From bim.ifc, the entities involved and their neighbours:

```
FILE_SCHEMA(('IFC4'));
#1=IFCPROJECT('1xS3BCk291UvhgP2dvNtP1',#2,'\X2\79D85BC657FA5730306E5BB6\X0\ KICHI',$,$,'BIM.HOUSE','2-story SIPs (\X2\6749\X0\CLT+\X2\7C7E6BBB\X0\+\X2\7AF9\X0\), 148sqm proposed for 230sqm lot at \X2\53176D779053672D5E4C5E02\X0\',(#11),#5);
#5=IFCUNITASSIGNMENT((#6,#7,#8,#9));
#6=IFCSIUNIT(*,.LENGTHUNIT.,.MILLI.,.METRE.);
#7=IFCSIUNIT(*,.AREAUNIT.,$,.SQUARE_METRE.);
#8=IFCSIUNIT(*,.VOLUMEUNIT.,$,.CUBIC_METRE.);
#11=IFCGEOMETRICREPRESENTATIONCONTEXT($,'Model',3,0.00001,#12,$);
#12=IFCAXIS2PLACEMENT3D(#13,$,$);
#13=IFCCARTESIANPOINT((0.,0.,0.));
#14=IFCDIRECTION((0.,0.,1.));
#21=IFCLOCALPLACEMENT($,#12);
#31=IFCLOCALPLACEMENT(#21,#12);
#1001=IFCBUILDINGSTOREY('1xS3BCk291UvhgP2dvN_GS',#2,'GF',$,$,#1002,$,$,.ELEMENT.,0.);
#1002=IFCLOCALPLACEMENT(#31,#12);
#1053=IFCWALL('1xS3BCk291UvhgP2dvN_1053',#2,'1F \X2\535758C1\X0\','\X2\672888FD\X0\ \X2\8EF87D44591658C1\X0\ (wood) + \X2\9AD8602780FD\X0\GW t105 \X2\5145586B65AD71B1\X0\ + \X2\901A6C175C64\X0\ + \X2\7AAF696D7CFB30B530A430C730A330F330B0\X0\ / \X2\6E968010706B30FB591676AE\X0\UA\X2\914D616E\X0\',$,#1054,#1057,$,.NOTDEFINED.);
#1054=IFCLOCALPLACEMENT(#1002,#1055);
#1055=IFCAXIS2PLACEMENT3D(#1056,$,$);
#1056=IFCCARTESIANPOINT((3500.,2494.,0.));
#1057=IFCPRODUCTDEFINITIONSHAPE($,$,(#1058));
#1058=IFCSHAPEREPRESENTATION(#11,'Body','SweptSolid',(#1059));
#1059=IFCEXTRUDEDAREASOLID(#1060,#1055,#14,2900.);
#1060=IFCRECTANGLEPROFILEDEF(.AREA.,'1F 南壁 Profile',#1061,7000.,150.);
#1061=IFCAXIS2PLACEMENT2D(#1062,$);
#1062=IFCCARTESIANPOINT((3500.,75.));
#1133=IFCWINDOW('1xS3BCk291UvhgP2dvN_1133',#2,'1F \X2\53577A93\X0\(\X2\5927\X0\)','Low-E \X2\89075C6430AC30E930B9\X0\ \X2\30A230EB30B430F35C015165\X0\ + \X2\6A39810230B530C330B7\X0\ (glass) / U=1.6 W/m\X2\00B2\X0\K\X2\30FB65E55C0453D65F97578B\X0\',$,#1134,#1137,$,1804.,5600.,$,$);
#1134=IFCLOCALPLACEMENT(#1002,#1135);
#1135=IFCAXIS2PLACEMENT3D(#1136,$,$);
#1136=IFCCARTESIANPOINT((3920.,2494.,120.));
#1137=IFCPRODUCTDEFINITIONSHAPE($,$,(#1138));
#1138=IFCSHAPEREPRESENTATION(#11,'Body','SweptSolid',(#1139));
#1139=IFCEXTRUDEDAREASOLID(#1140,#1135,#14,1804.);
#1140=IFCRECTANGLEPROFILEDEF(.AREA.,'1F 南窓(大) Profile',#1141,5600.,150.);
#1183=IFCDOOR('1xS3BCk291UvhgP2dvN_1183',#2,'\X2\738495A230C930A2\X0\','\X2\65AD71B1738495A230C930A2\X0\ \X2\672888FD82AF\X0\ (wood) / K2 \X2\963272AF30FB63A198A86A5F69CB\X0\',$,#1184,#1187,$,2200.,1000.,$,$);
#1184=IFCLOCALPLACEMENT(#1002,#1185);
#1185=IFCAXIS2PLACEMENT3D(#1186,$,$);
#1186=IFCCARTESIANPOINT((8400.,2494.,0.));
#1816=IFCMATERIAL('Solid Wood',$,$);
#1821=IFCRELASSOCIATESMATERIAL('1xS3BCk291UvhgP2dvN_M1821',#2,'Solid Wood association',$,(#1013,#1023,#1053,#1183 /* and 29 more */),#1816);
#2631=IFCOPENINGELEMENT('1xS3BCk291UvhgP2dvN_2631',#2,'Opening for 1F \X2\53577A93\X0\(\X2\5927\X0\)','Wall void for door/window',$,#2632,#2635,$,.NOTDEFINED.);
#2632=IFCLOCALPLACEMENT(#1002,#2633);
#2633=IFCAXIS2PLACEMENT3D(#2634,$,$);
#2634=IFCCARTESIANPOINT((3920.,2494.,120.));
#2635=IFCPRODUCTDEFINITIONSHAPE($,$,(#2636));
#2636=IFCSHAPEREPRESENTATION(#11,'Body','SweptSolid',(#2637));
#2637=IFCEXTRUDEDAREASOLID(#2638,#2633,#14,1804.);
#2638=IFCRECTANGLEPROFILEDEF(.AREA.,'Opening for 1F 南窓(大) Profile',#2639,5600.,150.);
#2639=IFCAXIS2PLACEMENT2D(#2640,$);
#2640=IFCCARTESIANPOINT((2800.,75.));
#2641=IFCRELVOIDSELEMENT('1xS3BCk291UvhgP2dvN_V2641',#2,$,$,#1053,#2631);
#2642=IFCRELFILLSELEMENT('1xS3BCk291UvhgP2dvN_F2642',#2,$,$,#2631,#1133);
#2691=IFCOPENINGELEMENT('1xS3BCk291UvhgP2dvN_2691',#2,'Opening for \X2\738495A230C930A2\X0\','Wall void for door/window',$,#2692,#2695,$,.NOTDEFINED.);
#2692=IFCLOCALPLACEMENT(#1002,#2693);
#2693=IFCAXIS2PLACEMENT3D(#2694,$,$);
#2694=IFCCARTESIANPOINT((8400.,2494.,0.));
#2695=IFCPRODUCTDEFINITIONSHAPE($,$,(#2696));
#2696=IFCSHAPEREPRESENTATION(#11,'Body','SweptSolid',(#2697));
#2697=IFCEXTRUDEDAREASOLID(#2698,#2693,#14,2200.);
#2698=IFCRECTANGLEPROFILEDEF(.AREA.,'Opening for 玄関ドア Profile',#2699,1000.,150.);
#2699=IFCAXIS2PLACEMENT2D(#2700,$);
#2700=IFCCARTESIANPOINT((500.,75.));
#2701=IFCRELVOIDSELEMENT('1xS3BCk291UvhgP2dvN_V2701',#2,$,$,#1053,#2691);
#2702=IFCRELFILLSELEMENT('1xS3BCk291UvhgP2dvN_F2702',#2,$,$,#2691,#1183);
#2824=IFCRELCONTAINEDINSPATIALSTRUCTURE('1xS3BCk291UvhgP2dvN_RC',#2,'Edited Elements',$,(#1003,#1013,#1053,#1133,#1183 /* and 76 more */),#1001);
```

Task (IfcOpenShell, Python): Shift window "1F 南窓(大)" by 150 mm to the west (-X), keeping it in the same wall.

```python
import ifcopenshell
import ifcopenshell.api.geometry
import ifcopenshell.util.placement
import ifcopenshell.util.unit

model = ifcopenshell.open("bim.ifc")
unit_scale = ifcopenshell.util.unit.calculate_unit_scale(model)

window = model.by_guid("1xS3BCk291UvhgP2dvN_1133")
opening = window.FillsVoids[0].RelatingOpeningElement
wall = opening.VoidsElements[0].RelatingBuildingElement

wall_matrix = ifcopenshell.util.placement.get_local_placement(wall.ObjectPlacement)
shift = wall_matrix[:3, 0] * -0.15 / unit_scale
before = ifcopenshell.util.placement.get_local_placement(window.ObjectPlacement)[:3, 3].copy()

# The window is not placed relative to its opening, so move both.
for product in (opening, window):
    matrix = ifcopenshell.util.placement.get_local_placement(product.ObjectPlacement)
    matrix[:3, 3] += shift
    ifcopenshell.api.geometry.edit_object_placement(model, product=product, matrix=matrix, is_si=False)

after = ifcopenshell.util.placement.get_local_placement(window.ObjectPlacement)[:3, 3]
print("window moved by", (after - before).round(3) + 0.0)

model.write("bim_v2.ifc")
```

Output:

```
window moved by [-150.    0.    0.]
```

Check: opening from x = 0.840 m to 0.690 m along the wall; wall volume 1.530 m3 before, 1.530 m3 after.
